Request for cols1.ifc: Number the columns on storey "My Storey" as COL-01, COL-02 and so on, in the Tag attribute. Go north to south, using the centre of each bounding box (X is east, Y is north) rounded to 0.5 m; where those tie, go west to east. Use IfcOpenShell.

First a look at what the model holds.

```python
import ifcopenshell
import ifcopenshell.util.element
import ifcopenshell.util.placement

model = ifcopenshell.open("cols1.ifc")
print(model.schema)
storey = next(s for s in model.by_type("IfcBuildingStorey") if s.Name == "My Storey")
columns = [e for e in ifcopenshell.util.element.get_decomposition(storey) if e.is_a("IfcColumn")]
for e in sorted(columns, key=lambda e: e.id()):
    origin = ifcopenshell.util.placement.get_local_placement(e.ObjectPlacement)[:3, 3]
    print(e.id(), e.Tag, e.Name, origin.round(2) + 0.0, sep=" | ")
```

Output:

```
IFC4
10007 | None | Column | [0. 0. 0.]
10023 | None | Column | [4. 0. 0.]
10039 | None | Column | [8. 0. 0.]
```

```python
import ifcopenshell
import ifcopenshell.geom
import ifcopenshell.util.element
import ifcopenshell.util.shape

model = ifcopenshell.open("cols1.ifc")
settings = ifcopenshell.geom.settings()
settings.set("use-world-coords", True)


def centre(element):
    shape = ifcopenshell.geom.create_shape(settings, element)
    return ifcopenshell.util.shape.get_bbox_centroid(shape.geometry)


storey = next(s for s in model.by_type("IfcBuildingStorey") if s.Name == "My Storey")
columns = [e for e in ifcopenshell.util.element.get_decomposition(storey) if e.is_a("IfcColumn")]

# Insertion points can sit at a corner or the storey origin, so sort by the geometry (in metres).
centres = {e: centre(e) for e in columns}
columns.sort(key=lambda e: (-round(centres[e][1] / 0.5), centres[e][0]))

for i, e in enumerate(columns, start=1):
    number = f"COL-{i:02d}"
    e.Tag = number
    print(e.id(), number)

model.write("cols1-out.ifc")
```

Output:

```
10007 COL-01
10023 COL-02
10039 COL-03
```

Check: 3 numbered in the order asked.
